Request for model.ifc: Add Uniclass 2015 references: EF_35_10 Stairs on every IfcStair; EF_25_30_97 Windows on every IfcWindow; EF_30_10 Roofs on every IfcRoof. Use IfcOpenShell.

First a look at what the model holds.

```python
import ifcopenshell

model = ifcopenshell.open("model.ifc")
print(model.schema)
print("classifications:", [c.Name for c in model.by_type("IfcClassification")])
for ifc_class in ("IfcDoor", "IfcRoof", "IfcStair", "IfcWall", "IfcWindow"):
    print(ifc_class, len(model.by_type(ifc_class)))
```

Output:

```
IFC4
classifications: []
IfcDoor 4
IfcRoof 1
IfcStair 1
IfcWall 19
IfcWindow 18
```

```python
import ifcopenshell
import ifcopenshell.api.classification

model = ifcopenshell.open("model.ifc")

system = ifcopenshell.api.classification.add_classification(model, classification="Uniclass 2015")

codes = {
    "IfcStair": ("EF_35_10", "Stairs"),
    "IfcWindow": ("EF_25_30_97", "Windows"),
    "IfcRoof": ("EF_30_10", "Roofs"),
}
for ifc_class, (code, name) in codes.items():
    products = model.by_type(ifc_class)
    ifcopenshell.api.classification.add_reference(
        model, products=products, classification=system, identification=code, name=name
    )
    print(code, len(products))

model.write("model_v2.ifc")
```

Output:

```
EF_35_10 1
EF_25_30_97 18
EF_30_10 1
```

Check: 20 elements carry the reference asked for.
